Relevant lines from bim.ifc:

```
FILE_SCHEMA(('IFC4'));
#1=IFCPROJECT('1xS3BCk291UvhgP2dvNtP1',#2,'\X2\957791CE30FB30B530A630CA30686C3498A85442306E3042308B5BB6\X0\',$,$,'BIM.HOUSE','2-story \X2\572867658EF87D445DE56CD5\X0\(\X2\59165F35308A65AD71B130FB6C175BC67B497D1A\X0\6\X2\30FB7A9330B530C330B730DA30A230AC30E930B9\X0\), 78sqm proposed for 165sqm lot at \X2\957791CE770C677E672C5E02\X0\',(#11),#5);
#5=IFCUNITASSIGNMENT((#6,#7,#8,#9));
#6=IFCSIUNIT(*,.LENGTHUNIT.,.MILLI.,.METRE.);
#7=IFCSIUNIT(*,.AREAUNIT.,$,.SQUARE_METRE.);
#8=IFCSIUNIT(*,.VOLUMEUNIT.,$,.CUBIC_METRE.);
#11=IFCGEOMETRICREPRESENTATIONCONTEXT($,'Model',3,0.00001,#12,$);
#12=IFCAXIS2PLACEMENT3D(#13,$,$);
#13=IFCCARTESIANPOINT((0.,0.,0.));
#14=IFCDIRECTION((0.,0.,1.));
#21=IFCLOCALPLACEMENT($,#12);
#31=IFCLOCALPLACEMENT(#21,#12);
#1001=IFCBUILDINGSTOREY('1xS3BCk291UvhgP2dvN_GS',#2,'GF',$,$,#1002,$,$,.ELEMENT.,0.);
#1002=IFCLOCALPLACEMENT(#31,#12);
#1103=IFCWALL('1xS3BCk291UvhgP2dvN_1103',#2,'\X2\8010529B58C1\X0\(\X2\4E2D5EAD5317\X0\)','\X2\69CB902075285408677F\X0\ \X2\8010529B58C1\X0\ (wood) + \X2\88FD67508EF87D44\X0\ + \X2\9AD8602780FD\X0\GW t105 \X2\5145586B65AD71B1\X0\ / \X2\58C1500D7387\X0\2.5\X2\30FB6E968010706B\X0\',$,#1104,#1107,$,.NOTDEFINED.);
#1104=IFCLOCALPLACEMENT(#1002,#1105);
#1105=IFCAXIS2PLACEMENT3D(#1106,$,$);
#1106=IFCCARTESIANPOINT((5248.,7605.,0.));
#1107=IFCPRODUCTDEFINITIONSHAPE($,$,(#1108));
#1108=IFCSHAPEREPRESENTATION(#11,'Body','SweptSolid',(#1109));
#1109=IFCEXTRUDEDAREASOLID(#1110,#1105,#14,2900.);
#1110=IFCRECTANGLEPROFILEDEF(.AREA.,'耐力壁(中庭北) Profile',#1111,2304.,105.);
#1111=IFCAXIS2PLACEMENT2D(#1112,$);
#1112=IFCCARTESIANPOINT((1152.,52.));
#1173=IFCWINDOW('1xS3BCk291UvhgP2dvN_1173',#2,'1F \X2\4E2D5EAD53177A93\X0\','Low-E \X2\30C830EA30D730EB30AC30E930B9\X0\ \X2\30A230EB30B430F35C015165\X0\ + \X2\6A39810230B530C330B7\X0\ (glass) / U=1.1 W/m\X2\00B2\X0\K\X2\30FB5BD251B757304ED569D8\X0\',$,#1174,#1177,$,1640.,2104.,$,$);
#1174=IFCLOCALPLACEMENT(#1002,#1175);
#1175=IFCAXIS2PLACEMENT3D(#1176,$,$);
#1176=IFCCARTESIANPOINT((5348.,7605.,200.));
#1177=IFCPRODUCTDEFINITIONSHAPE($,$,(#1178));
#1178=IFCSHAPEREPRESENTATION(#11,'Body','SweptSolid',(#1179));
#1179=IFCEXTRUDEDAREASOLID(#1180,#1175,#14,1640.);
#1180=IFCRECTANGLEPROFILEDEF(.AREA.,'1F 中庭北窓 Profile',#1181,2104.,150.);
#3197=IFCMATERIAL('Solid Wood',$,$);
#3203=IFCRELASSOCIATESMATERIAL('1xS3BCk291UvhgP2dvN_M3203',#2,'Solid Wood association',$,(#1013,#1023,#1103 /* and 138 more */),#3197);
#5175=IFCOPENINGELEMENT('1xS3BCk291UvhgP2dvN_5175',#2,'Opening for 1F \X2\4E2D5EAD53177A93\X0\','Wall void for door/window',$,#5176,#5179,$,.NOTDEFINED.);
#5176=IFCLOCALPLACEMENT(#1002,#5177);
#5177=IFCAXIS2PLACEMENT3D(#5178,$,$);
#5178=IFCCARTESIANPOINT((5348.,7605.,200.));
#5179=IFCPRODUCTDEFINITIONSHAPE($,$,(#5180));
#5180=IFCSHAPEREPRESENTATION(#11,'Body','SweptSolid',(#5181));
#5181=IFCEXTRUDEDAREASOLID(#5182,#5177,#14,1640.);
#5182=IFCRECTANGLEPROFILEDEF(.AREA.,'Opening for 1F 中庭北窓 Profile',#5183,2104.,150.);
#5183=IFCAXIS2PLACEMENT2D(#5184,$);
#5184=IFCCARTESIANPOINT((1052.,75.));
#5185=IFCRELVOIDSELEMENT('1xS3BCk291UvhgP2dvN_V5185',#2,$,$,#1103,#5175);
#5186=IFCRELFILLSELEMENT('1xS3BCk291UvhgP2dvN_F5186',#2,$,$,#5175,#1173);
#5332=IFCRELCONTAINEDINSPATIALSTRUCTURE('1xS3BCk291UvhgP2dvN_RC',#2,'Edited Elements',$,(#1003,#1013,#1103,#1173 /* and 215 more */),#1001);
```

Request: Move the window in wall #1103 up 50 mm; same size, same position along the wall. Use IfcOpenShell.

```python
import numpy as np
import ifcopenshell
import ifcopenshell.api.geometry
import ifcopenshell.util.placement
import ifcopenshell.util.unit

model = ifcopenshell.open("bim.ifc")
unit_scale = ifcopenshell.util.unit.calculate_unit_scale(model)

window = model.by_id(1173)
opening = window.FillsVoids[0].RelatingOpeningElement
dz = 50.0

shift = np.array([0.0, 0.0, dz])
# The window is not placed relative to its opening, so move both.
for product in (opening, window):
    matrix = ifcopenshell.util.placement.get_local_placement(product.ObjectPlacement)
    matrix[:3, 3] += shift
    ifcopenshell.api.geometry.edit_object_placement(model, product=product, matrix=matrix, is_si=False)

print(f"moved by {dz * unit_scale:+.3f} m")

model.write("bim_rev.ifc")
```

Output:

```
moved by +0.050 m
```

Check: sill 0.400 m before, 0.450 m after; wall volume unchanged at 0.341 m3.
